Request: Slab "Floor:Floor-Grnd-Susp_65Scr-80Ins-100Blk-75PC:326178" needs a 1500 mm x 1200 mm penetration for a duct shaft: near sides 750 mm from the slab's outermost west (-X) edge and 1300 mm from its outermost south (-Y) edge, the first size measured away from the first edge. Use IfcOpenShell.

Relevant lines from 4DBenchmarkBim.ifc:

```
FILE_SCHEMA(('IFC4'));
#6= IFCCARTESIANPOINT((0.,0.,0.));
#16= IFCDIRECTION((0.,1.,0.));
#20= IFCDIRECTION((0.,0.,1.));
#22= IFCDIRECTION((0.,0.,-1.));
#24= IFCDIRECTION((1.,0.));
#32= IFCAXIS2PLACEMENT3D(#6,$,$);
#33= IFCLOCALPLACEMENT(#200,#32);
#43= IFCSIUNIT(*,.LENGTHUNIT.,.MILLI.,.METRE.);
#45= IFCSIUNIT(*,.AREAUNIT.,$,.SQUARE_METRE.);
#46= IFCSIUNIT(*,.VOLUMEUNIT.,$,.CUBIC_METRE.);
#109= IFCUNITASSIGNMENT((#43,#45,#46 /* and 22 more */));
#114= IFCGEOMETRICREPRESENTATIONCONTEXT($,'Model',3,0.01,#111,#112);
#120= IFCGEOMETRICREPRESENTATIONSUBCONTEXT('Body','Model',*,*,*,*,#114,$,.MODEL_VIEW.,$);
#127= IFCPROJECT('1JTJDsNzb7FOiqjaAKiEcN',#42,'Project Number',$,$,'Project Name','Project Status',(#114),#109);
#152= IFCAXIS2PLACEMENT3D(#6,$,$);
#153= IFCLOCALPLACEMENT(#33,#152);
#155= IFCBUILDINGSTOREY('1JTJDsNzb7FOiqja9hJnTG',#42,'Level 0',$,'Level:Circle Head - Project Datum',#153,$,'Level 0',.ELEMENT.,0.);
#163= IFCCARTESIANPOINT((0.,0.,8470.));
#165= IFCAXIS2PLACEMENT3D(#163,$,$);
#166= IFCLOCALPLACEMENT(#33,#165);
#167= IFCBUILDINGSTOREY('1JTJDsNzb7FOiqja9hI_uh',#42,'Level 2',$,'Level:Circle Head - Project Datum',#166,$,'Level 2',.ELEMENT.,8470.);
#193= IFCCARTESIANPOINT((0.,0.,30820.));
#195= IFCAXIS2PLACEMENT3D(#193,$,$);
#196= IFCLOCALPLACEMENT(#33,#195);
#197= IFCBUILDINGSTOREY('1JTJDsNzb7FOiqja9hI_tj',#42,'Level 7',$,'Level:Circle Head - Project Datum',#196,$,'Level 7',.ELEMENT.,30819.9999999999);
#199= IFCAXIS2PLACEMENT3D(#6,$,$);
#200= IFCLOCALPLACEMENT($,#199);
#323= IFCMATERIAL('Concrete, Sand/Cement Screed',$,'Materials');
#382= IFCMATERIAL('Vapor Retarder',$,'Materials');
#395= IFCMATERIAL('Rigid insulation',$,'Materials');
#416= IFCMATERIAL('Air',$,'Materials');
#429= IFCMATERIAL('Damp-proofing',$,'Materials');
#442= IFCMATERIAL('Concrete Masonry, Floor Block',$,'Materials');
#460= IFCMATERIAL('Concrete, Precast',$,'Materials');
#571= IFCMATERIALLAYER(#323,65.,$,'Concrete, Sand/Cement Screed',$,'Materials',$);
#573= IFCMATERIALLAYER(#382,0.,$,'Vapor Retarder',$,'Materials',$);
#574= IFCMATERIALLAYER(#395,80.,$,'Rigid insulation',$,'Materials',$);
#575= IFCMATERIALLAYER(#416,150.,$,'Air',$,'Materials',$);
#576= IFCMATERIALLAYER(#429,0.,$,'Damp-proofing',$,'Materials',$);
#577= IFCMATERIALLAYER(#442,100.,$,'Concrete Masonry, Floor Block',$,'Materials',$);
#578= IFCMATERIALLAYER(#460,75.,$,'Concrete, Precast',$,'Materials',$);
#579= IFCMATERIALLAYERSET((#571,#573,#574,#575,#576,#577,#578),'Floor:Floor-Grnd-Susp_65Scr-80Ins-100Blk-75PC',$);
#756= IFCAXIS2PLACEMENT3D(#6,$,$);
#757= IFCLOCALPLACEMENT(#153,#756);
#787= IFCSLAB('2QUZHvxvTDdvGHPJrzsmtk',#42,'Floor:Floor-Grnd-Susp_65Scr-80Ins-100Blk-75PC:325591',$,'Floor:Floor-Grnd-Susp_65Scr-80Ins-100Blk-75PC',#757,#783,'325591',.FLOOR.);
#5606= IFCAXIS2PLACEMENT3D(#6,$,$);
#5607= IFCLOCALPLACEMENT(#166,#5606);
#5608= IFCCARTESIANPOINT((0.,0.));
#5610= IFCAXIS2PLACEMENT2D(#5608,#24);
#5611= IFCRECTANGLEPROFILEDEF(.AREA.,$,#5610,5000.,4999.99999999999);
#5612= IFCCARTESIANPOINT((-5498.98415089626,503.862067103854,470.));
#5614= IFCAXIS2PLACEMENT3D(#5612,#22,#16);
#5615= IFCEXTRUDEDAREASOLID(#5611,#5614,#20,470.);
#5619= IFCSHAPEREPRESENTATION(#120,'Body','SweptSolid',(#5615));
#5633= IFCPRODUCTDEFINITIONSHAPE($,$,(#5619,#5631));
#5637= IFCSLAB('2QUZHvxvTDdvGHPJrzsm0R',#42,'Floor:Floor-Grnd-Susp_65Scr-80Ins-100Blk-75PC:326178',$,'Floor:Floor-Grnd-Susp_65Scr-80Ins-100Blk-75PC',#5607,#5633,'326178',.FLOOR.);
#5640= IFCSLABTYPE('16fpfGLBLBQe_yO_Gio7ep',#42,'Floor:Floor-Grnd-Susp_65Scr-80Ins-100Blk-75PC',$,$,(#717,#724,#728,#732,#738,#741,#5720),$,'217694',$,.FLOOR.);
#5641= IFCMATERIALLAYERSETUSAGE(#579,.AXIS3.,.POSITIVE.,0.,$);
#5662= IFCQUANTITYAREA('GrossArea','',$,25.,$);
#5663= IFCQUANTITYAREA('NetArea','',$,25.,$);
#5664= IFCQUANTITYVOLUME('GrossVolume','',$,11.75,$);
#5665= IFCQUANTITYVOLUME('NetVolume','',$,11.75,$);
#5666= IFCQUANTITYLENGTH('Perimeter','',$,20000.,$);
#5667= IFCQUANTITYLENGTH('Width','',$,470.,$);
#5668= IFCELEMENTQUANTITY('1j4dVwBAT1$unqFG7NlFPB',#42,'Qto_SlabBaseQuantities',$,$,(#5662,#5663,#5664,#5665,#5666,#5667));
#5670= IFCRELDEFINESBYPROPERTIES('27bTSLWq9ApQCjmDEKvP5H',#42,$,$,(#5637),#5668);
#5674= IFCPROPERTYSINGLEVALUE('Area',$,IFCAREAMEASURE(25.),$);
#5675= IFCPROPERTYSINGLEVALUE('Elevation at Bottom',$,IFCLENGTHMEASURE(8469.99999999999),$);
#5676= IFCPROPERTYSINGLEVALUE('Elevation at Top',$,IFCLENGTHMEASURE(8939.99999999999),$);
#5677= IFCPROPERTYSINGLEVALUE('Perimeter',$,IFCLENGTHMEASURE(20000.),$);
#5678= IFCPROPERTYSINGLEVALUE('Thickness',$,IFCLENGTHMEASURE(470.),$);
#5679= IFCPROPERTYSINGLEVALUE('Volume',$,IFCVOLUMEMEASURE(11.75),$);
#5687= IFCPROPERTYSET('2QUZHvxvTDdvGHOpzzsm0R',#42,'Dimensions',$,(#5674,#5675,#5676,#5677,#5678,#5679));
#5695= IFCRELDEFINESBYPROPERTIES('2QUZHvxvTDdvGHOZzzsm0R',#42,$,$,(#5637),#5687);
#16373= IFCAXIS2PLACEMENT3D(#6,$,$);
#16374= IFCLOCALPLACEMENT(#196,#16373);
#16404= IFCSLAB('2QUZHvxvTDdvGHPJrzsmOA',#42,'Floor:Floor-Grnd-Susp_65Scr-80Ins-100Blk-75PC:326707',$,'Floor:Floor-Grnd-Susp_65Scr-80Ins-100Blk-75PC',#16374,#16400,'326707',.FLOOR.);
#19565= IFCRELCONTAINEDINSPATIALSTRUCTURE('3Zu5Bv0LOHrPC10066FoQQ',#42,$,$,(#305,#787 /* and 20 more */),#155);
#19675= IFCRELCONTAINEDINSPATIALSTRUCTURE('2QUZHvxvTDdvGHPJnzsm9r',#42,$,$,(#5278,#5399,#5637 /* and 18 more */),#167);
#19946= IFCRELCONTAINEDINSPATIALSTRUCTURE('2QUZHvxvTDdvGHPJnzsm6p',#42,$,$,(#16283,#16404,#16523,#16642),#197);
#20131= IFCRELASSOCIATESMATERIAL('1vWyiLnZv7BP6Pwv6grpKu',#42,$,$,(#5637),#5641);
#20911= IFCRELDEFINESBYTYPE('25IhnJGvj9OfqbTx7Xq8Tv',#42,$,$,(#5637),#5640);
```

```python
import numpy as np
import ifcopenshell
import ifcopenshell.api.feature
import ifcopenshell.api.geometry
import ifcopenshell.api.pset
import ifcopenshell.api.root
import ifcopenshell.geom
import ifcopenshell.util.element
import ifcopenshell.util.placement
import ifcopenshell.util.representation
import ifcopenshell.util.shape
import ifcopenshell.util.unit

model = ifcopenshell.open("4DBenchmarkBim.ifc")
unit_scale = ifcopenshell.util.unit.calculate_unit_scale(model)
area_scale = ifcopenshell.util.unit.calculate_unit_scale(model, "AREAUNIT")
volume_scale = ifcopenshell.util.unit.calculate_unit_scale(model, "VOLUMEUNIT")
settings = ifcopenshell.geom.settings()


def volume(element):
    """Net volume in cubic metres, openings subtracted."""
    shape = ifcopenshell.geom.create_shape(settings, element)
    return ifcopenshell.util.shape.get_volume(shape.geometry)


slab = model.by_guid("2QUZHvxvTDdvGHPJrzsm0R")
before = volume(slab)

# Extent in the slab's own axes, in metres. The edges named are its -X and -Y sides.
slab_shape = ifcopenshell.geom.create_shape(settings, slab)
vertices = ifcopenshell.util.shape.get_vertices(slab_shape.geometry)
x_min, y_min, bottom = vertices.min(axis=0)
top = vertices[:, 2].max()

opening = ifcopenshell.api.root.create_entity(model, ifc_class="IfcOpeningElement", name="Duct shaft opening", predefined_type="OPENING")
context = ifcopenshell.util.representation.get_context(model, "Model", "Body", "MODEL_VIEW")
width, depth = 1.5, 1.2
outline = [(0.0, 0.0), (width, 0.0), (width, depth), (0.0, depth), (0.0, 0.0)]
# Overshoot both faces by 50 mm so the cut is clean.
shape = ifcopenshell.api.geometry.add_slab_representation(
    model, context=context, depth=top - bottom + 0.1, polyline=outline
)
ifcopenshell.api.geometry.assign_representation(model, product=opening, representation=shape)

matrix = ifcopenshell.util.placement.get_local_placement(slab.ObjectPlacement)
matrix[:, 3] = matrix @ np.append(np.array([x_min + 0.75, y_min + 1.3, bottom - 0.05]) / unit_scale, 1.0)
ifcopenshell.api.geometry.edit_object_placement(model, product=opening, matrix=matrix, is_si=False)
ifcopenshell.api.feature.add_feature(model, feature=opening, element=slab)

after = volume(slab)

# Update the slab's stored quantities.
qto = model.by_id(ifcopenshell.util.element.get_pset(slab, "Qto_SlabBaseQuantities", should_inherit=False)["id"])
ifcopenshell.api.pset.edit_qto(model, qto=qto, properties={
    "NetArea": after / (top - bottom) / area_scale,
    "NetVolume": after / volume_scale,
})
pset = model.by_id(ifcopenshell.util.element.get_pset(slab, "Dimensions", should_inherit=False)["id"])
ifcopenshell.api.pset.edit_pset(model, pset=pset, properties={
    "Area": model.create_entity("IfcAreaMeasure", after / (top - bottom) / area_scale),
    "Volume": model.create_entity("IfcVolumeMeasure", after / volume_scale),
})

print(f"slab volume {before:.3f} -> {after:.3f} m3")

model.write("4DBenchmarkBim-out.ifc")
```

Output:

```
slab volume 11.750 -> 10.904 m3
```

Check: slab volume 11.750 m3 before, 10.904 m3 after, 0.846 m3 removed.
